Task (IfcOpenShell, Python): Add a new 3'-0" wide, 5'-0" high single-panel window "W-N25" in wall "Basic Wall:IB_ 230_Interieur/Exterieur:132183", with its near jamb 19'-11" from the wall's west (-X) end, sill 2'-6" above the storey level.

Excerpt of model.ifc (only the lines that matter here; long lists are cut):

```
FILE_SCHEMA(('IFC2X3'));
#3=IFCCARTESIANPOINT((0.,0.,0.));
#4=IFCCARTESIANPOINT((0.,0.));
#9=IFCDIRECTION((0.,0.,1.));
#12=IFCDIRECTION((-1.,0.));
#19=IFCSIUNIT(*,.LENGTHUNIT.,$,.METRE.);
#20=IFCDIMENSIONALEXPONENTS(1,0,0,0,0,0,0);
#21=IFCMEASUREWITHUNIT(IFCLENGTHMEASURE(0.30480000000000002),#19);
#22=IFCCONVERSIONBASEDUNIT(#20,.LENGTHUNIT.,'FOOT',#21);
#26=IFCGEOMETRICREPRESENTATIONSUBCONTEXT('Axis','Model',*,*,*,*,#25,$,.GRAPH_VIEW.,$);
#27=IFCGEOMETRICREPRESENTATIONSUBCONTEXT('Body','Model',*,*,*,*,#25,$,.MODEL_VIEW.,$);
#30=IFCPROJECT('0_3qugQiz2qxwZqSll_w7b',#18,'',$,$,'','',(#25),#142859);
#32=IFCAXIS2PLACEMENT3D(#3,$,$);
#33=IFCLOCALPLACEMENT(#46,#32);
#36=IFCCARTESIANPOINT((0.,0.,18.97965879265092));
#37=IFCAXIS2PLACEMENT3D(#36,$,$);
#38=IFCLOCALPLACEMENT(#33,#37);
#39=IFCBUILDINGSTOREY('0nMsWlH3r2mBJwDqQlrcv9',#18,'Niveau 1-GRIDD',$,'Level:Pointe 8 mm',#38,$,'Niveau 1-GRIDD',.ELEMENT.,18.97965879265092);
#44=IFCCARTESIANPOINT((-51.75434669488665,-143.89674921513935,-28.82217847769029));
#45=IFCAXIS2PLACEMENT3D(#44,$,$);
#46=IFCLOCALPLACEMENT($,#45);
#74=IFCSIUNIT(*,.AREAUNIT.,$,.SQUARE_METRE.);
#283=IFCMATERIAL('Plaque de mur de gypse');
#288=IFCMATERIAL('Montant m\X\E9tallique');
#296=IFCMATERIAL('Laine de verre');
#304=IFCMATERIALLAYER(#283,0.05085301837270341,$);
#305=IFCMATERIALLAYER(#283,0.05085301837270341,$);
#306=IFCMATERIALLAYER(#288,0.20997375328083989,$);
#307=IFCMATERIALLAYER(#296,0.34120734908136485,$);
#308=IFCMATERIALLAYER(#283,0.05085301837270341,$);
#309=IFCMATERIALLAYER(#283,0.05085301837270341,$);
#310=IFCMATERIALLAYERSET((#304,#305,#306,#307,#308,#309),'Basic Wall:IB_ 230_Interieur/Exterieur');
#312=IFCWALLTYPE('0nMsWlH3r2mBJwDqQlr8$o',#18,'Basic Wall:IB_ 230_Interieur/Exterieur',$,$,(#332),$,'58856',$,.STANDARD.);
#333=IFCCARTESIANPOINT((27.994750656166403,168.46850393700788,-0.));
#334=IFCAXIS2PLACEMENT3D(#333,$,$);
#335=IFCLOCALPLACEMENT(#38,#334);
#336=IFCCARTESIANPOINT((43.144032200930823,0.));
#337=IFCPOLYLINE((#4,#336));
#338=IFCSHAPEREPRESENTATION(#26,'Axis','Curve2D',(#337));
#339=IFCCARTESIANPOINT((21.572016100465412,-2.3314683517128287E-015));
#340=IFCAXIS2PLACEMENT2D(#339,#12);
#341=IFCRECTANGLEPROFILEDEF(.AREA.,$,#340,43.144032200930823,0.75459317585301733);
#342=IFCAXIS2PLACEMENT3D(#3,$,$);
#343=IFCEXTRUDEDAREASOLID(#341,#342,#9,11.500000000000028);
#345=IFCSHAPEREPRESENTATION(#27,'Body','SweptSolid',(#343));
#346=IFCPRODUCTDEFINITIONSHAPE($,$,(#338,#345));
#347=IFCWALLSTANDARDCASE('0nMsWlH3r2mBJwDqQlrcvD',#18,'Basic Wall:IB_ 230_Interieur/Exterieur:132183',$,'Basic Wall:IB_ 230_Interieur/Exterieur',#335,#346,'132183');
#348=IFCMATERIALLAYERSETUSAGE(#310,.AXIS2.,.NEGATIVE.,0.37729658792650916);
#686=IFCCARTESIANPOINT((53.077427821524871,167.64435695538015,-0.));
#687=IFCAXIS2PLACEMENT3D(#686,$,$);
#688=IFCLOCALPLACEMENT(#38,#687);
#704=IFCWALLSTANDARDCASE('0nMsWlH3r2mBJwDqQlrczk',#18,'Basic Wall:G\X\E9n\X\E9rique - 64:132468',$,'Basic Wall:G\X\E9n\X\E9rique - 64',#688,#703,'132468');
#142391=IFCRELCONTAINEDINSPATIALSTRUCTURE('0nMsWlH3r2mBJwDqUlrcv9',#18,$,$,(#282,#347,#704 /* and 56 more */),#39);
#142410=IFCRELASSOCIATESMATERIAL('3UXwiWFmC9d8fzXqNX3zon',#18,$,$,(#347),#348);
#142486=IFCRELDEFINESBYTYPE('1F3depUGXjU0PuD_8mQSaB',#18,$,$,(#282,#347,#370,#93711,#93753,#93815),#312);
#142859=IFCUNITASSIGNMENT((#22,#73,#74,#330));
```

```python
import numpy as np
import ifcopenshell
import ifcopenshell.api.feature
import ifcopenshell.api.geometry
import ifcopenshell.api.root
import ifcopenshell.api.spatial
import ifcopenshell.api.type
import ifcopenshell.geom
import ifcopenshell.util.element
import ifcopenshell.util.placement
import ifcopenshell.util.representation
import ifcopenshell.util.shape
import ifcopenshell.util.unit

model = ifcopenshell.open("model.ifc")
unit_scale = ifcopenshell.util.unit.calculate_unit_scale(model)
settings = ifcopenshell.geom.settings()


def volume(element):
    """Net volume in cubic metres, openings subtracted."""
    shape = ifcopenshell.geom.create_shape(settings, element)
    return ifcopenshell.util.shape.get_volume(shape.geometry)


wall = model.by_guid("0nMsWlH3r2mBJwDqQlrcvD")
storey = ifcopenshell.util.element.get_container(wall, ifc_class="IfcBuildingStorey")
context = ifcopenshell.util.representation.get_context(model, "Model", "Body", "MODEL_VIEW")
before = volume(wall)

width, height, from_end, sill = 0.9144, 1.524, 6.0706, 0.762  # metres

# The wall runs along its own X axis, and the end named is its -X end.
wall_shape = ifcopenshell.geom.create_shape(settings, wall)
x, y, z = ifcopenshell.util.shape.get_vertices(wall_shape.geometry).T
start = x.min() + from_end
face, thickness = float(y.min()), float(y.max() - y.min())
wall_matrix = ifcopenshell.util.placement.get_local_placement(wall.ObjectPlacement)
level = ifcopenshell.util.placement.get_local_placement(storey.ObjectPlacement)[2, 3]


def in_wall(x, y):
    """Placement at x, y metres in the wall's axes, at sill height."""
    matrix = wall_matrix.copy()
    matrix[:, 3] = wall_matrix @ np.array([x / unit_scale, y / unit_scale, 0.0, 1.0])
    matrix[2, 3] = level + sill / unit_scale
    return matrix


# Opening: a box that overshoots both wall faces by 50 mm.
opening = ifcopenshell.api.root.create_entity(model, ifc_class="IfcOpeningElement")
box = ifcopenshell.api.geometry.add_wall_representation(
    model, context=context, length=width, height=height, thickness=thickness + 0.1
)
ifcopenshell.api.geometry.assign_representation(model, product=opening, representation=box)
ifcopenshell.api.geometry.edit_object_placement(model, product=opening, matrix=in_wall(start, face - 0.05), is_si=False)
ifcopenshell.api.feature.add_feature(model, feature=opening, element=wall)

window = ifcopenshell.api.root.create_entity(model, ifc_class="IfcWindow", name="W-N25")
window.OverallWidth, window.OverallHeight = width / unit_scale, height / unit_scale
body = ifcopenshell.api.geometry.add_window_representation(
    model,
    context=context,
    overall_width=window.OverallWidth,
    overall_height=window.OverallHeight,
    partition_type="SINGLE_PANEL",
)
ifcopenshell.api.geometry.assign_representation(model, product=window, representation=body)
ifcopenshell.api.spatial.assign_container(model, products=[window], relating_structure=storey)
fills = ifcopenshell.api.feature.add_filling(model, opening=opening, element=window)
fills.OwnerHistory = window.OwnerHistory  # required in IFC2X3

# IFC2X3 keeps the operation on the window style.
style = ifcopenshell.api.root.create_entity(model, ifc_class="IfcWindowStyle", name="W-N25")
style.OperationType, style.ConstructionType = "SINGLE_PANEL", "NOTDEFINED"
style.ParameterTakesPrecedence = style.Sizeable = False
ifcopenshell.api.type.assign_type(model, related_objects=[window], relating_type=style)

# Centre the window in the wall's thickness.
ifcopenshell.api.geometry.edit_object_placement(model, product=window, matrix=in_wall(start, face), is_si=False)
window_shape = ifcopenshell.geom.create_shape(settings, window)
depth = ifcopenshell.util.shape.get_vertices(window_shape.geometry)[:, 1]
offset = face + thickness / 2 - (depth.min() + depth.max()) / 2
ifcopenshell.api.geometry.edit_object_placement(model, product=window, matrix=in_wall(start, offset), is_si=False)

after = volume(wall)

print(f"wall volume {before:.3f} -> {after:.3f} m3")

model.write("model_v2.ifc")
```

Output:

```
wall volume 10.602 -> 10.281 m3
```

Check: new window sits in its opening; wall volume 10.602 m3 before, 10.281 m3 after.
